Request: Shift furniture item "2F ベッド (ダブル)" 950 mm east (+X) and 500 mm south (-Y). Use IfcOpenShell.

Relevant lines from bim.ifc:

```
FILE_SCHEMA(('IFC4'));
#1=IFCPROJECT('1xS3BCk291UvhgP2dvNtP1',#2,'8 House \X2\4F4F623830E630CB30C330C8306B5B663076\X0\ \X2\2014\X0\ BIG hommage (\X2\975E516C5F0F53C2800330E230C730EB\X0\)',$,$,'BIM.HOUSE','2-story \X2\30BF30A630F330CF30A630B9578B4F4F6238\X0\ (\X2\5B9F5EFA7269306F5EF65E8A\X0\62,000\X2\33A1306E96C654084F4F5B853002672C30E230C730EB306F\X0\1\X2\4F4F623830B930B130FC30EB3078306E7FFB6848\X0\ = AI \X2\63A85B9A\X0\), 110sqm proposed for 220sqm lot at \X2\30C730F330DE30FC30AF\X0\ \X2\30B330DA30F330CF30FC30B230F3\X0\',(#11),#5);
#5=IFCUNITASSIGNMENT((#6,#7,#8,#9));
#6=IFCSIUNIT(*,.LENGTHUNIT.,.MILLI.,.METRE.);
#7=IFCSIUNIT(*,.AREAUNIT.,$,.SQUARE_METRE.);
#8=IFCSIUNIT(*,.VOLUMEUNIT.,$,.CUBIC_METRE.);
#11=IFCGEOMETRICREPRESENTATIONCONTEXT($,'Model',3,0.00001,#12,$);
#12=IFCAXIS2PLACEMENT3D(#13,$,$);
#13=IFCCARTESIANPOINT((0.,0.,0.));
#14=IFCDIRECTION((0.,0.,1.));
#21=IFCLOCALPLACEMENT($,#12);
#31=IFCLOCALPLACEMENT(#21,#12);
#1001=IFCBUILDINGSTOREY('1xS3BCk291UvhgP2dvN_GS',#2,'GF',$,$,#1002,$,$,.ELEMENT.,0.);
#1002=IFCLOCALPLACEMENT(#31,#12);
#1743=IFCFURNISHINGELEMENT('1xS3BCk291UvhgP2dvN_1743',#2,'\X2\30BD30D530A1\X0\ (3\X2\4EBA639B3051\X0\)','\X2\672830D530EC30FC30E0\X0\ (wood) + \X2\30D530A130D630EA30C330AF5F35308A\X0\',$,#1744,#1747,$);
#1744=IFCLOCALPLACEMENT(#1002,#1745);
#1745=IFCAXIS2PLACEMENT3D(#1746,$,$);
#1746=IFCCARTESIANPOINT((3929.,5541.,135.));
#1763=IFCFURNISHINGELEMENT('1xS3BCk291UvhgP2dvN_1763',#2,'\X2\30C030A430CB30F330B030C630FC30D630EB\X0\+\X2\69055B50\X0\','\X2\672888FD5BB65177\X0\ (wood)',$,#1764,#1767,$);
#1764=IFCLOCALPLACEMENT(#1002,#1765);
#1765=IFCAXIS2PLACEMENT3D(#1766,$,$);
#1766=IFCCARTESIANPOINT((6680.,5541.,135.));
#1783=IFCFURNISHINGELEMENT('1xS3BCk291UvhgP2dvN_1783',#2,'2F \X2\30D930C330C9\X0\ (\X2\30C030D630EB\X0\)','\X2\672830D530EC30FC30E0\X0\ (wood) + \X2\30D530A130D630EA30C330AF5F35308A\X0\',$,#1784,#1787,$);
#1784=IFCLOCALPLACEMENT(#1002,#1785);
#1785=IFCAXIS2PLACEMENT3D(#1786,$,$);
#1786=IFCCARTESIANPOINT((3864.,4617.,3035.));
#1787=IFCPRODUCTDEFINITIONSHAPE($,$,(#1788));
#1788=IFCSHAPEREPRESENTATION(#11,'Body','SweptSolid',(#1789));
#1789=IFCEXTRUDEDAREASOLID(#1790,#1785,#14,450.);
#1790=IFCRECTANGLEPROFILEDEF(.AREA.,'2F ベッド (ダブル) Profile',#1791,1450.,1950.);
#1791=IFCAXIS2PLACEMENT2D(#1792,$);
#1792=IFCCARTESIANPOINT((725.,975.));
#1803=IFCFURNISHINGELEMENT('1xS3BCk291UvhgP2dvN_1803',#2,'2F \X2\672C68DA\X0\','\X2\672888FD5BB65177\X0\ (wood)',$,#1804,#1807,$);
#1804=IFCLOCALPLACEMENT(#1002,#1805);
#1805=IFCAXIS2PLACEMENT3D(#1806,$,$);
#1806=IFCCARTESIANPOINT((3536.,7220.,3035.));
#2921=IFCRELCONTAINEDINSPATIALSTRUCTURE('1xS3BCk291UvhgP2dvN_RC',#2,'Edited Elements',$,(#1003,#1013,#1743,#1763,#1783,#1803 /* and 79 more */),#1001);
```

```python
import ifcopenshell
import ifcopenshell.api.geometry
import ifcopenshell.util.placement
import ifcopenshell.util.unit

model = ifcopenshell.open("bim.ifc")
unit_scale = ifcopenshell.util.unit.calculate_unit_scale(model)

item = model.by_guid("1xS3BCk291UvhgP2dvN_1783")
matrix = ifcopenshell.util.placement.get_local_placement(item.ObjectPlacement)
matrix[0, 3] += 0.95 / unit_scale
matrix[1, 3] -= 0.5 / unit_scale
ifcopenshell.api.geometry.edit_object_placement(model, product=item, matrix=matrix, is_si=False)

print(ifcopenshell.util.placement.get_local_placement(item.ObjectPlacement).round(3) + 0.0)

model.write("bim_edited.ifc")
```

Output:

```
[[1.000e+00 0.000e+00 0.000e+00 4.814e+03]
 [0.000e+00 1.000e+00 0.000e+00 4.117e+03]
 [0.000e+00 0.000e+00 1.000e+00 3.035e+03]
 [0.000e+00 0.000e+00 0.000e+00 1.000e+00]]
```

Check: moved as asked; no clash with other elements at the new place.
